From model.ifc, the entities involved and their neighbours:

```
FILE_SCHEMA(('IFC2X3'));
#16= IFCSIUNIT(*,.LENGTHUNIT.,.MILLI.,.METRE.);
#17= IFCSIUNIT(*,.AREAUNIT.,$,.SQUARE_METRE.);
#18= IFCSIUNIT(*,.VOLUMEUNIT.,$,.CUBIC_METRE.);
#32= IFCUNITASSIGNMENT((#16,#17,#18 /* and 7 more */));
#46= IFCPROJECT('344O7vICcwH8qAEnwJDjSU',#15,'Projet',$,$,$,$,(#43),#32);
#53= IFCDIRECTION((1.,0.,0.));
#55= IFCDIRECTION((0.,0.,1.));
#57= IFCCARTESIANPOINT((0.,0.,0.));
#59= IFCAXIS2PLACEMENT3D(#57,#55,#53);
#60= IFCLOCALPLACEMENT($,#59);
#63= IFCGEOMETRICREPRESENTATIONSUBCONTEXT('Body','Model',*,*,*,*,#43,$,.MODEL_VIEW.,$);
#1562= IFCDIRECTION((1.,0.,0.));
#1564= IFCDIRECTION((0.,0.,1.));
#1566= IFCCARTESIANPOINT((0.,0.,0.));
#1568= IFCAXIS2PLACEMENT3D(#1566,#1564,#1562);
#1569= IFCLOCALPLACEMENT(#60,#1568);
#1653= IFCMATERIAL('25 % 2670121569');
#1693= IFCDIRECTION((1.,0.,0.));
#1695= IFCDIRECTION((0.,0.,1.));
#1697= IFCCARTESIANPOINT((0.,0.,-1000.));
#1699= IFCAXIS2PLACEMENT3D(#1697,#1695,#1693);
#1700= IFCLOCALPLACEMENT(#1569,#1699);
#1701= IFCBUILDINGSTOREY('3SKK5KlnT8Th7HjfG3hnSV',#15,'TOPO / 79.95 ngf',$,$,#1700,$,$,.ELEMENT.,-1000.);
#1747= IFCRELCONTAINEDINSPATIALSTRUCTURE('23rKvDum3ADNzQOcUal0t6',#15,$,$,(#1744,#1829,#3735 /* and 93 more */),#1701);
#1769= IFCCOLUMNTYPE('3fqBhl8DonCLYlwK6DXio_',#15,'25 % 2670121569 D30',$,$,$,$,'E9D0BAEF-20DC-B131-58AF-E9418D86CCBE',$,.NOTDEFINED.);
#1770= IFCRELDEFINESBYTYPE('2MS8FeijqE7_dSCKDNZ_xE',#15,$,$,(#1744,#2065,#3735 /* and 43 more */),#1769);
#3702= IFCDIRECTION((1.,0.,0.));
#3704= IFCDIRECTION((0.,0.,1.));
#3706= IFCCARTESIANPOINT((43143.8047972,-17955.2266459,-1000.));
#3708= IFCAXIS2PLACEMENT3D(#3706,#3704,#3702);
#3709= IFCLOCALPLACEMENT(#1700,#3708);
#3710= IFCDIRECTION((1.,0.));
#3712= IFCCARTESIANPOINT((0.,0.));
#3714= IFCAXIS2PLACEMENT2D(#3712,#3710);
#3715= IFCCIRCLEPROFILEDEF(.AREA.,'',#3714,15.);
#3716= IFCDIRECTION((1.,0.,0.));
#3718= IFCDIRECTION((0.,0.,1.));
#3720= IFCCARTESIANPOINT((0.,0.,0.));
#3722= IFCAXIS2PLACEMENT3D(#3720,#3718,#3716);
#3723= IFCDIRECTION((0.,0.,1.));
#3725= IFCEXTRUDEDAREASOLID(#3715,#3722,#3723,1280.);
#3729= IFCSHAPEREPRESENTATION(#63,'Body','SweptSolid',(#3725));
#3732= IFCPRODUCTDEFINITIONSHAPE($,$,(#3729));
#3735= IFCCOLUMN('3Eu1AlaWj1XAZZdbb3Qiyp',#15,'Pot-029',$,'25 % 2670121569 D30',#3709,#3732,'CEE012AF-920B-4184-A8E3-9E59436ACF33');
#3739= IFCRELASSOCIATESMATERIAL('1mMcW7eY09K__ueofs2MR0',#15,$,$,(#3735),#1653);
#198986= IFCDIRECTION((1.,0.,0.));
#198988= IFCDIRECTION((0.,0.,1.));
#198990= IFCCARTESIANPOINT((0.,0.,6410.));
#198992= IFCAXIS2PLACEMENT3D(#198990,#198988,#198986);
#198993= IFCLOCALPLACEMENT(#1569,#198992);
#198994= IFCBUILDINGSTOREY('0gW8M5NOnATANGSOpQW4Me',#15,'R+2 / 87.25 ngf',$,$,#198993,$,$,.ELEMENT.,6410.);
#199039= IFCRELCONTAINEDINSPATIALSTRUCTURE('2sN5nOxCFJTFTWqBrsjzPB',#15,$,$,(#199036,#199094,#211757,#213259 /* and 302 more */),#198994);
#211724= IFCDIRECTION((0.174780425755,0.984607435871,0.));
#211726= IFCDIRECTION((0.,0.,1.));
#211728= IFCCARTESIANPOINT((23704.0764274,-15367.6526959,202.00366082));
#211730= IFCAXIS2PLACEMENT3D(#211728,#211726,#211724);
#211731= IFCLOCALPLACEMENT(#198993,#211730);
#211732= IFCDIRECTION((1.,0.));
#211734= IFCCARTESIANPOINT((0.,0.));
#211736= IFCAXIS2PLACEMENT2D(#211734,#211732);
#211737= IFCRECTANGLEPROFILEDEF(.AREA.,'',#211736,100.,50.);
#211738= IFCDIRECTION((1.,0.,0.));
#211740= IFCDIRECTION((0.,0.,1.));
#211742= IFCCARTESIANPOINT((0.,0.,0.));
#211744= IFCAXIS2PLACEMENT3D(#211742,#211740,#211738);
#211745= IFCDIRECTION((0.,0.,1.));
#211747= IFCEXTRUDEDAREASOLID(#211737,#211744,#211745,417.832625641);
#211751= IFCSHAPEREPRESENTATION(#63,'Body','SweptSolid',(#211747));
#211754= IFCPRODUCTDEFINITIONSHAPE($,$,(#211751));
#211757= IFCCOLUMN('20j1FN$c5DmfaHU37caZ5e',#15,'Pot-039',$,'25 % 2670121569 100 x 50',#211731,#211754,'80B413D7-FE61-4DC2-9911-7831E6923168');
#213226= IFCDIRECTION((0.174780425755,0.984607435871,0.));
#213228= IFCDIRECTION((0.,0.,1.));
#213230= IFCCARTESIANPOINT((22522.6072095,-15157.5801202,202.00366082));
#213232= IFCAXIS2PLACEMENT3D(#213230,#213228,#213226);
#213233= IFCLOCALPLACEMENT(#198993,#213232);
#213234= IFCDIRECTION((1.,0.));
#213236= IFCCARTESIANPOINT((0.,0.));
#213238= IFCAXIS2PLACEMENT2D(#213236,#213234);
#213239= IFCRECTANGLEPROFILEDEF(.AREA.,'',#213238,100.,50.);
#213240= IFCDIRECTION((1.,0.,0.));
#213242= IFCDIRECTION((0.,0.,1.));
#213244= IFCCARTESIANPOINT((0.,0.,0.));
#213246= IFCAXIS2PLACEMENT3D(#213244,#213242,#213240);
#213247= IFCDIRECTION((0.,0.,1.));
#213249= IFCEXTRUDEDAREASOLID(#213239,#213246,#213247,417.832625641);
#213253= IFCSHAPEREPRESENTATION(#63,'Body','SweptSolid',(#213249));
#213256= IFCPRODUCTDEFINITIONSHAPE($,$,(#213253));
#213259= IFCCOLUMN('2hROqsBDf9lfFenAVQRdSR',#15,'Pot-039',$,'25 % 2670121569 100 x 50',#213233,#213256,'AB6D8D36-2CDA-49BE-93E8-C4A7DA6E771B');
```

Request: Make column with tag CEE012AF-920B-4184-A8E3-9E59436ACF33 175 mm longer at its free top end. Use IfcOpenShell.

```python
import ifcopenshell
import ifcopenshell.util.representation
import ifcopenshell.util.unit

model = ifcopenshell.open("model.ifc")
unit_scale = ifcopenshell.util.unit.calculate_unit_scale(model)

member = model.by_guid("3Eu1AlaWj1XAZZdbb3Qiyp")
change = 0.175 / unit_scale

# The extrusion runs towards the end named, so only its depth changes.
body = ifcopenshell.util.representation.get_representation(member, "Model", "Body")
solid = body.Items[0]
old_length = solid.Depth
solid.Depth += change

print(f"length {old_length:g} -> {solid.Depth:g}")

model.write("model_updated.ifc")
```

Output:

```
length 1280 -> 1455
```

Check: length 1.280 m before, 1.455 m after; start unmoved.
